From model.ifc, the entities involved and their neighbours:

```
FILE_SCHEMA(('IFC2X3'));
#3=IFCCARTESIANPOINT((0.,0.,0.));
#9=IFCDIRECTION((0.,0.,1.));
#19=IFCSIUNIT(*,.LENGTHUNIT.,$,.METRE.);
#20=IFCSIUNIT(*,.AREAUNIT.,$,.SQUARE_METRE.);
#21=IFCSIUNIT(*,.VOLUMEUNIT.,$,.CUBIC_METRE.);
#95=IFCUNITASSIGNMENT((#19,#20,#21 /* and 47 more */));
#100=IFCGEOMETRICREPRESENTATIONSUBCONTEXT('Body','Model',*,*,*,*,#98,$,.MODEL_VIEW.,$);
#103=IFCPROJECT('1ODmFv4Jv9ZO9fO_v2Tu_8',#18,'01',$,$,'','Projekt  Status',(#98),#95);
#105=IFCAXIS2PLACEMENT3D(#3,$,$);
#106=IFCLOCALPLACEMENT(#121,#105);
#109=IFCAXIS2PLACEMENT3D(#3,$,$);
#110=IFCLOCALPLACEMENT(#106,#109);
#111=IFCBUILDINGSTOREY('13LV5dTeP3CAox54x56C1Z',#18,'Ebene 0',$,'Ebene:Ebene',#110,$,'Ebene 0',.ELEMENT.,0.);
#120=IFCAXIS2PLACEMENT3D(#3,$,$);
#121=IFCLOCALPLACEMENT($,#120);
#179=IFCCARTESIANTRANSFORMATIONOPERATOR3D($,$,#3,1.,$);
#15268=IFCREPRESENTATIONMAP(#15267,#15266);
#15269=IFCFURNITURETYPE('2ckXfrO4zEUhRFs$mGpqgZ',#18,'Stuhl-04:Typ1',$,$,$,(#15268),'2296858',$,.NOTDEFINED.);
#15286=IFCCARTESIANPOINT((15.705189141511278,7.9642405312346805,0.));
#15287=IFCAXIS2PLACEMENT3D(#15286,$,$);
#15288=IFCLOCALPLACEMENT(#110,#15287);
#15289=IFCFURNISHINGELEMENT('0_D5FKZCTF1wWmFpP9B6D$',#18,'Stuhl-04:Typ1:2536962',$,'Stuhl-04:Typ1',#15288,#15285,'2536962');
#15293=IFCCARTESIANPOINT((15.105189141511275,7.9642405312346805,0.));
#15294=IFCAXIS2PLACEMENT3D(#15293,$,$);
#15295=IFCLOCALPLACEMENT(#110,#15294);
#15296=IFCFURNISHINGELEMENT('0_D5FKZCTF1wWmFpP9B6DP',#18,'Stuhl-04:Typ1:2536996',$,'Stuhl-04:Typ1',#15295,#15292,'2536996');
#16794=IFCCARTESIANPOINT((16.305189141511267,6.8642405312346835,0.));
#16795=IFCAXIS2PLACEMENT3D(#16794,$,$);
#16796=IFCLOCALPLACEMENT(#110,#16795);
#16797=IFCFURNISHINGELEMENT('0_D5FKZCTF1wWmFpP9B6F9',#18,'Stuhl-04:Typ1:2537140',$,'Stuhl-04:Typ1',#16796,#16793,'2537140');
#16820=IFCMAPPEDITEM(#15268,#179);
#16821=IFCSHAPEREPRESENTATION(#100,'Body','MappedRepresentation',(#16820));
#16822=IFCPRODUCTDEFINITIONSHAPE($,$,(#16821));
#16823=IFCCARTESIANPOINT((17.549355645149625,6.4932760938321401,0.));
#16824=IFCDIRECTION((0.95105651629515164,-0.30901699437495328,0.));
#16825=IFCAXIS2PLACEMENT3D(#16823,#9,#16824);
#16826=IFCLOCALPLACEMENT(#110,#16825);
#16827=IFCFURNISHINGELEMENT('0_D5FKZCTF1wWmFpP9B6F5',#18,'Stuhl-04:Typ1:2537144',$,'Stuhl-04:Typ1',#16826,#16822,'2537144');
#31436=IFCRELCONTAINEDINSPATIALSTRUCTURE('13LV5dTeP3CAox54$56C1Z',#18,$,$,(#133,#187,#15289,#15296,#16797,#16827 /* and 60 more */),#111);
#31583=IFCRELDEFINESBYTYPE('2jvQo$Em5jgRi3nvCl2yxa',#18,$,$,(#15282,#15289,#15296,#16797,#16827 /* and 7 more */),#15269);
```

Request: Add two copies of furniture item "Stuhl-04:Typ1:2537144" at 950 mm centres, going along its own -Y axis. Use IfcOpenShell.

```python
import ifcopenshell
import ifcopenshell.api.geometry
import ifcopenshell.api.root
import ifcopenshell.util.element
import ifcopenshell.util.placement
import ifcopenshell.util.unit

model = ifcopenshell.open("model.ifc")
unit_scale = ifcopenshell.util.unit.calculate_unit_scale(model)

source = model.by_guid("0_D5FKZCTF1wWmFpP9B6F5")
base = ifcopenshell.util.placement.get_local_placement(source.ObjectPlacement)
step = -base[:3, 1] * 0.95 / unit_scale

for i in range(1, 3):
    copy = ifcopenshell.api.root.copy_class(model, product=source)
    copy.Representation = ifcopenshell.util.element.copy_deep(
        model, source.Representation, exclude=["IfcGeometricRepresentationContext", "IfcRepresentationMap"]
    )
    copy.Name = "Stuhl-04:Typ1"
    copy.Tag = None
    matrix = base.copy()
    matrix[:3, 3] += i * step
    print("added at", matrix[:3, 3].round(3) + 0.0)
    ifcopenshell.api.geometry.edit_object_placement(model, product=copy, matrix=matrix, is_si=False)

model.write("model_rev.ifc")
```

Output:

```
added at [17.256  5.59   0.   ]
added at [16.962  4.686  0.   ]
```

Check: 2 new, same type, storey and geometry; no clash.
